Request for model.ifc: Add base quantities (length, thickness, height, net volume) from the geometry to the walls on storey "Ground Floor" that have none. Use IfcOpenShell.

First a look at what the model holds.

```python
import ifcopenshell
import ifcopenshell.util.element
import ifcopenshell.util.unit

model = ifcopenshell.open("model.ifc")
print(model.schema)
for unit_type in ("LENGTHUNIT", "AREAUNIT", "VOLUMEUNIT"):
    print(unit_type, ifcopenshell.util.unit.calculate_unit_scale(model, unit_type))
storey = next(s for s in model.by_type("IfcBuildingStorey") if s.Name == "Ground Floor")
walls = [e for e in ifcopenshell.util.element.get_decomposition(storey) if e.is_a("IfcWall")]
for e in sorted(walls, key=lambda e: e.id()):
    print(e.id(), e.is_a(), e.Name, list(ifcopenshell.util.element.get_psets(e, qtos_only=True)), sep=" | ")
```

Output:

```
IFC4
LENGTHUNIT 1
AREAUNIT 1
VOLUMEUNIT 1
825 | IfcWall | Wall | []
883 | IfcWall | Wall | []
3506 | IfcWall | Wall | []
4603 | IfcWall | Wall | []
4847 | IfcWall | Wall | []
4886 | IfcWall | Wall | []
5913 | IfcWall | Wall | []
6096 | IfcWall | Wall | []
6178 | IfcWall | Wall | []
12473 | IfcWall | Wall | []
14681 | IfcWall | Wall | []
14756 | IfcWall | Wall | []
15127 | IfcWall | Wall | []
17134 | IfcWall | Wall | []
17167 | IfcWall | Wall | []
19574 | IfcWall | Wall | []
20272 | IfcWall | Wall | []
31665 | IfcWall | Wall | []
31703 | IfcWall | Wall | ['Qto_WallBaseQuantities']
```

```python
import ifcopenshell
import ifcopenshell.api.pset
import ifcopenshell.geom
import ifcopenshell.util.element
import ifcopenshell.util.shape
import ifcopenshell.util.unit

model = ifcopenshell.open("model.ifc")
unit_scale = ifcopenshell.util.unit.calculate_unit_scale(model)
volume_scale = ifcopenshell.util.unit.calculate_unit_scale(model, "VOLUMEUNIT")
settings = ifcopenshell.geom.settings()

storey = next(s for s in model.by_type("IfcBuildingStorey") if s.Name == "Ground Floor")
walls = [e for e in ifcopenshell.util.element.get_decomposition(storey) if e.is_a("IfcWall")]

for e in sorted(walls, key=lambda e: e.id()):
    if ifcopenshell.util.element.get_psets(e, qtos_only=True, should_inherit=False):
        continue
    # Geometry comes back in metres, in the element's own axes.
    shape = ifcopenshell.geom.create_shape(settings, e)
    values = {
        "Length": ifcopenshell.util.shape.get_x(shape.geometry) / unit_scale,
        "Width": ifcopenshell.util.shape.get_y(shape.geometry) / unit_scale,
        "Height": ifcopenshell.util.shape.get_z(shape.geometry) / unit_scale,
        "NetVolume": ifcopenshell.util.shape.get_volume(shape.geometry) / volume_scale,
    }
    qto = ifcopenshell.api.pset.add_qto(model, product=e, name="Qto_WallBaseQuantities")
    ifcopenshell.api.pset.edit_qto(model, qto=qto, properties=values)
    print(e.id(), {k: round(v, 3) for k, v in values.items()})

model.write("model_updated.ifc")
```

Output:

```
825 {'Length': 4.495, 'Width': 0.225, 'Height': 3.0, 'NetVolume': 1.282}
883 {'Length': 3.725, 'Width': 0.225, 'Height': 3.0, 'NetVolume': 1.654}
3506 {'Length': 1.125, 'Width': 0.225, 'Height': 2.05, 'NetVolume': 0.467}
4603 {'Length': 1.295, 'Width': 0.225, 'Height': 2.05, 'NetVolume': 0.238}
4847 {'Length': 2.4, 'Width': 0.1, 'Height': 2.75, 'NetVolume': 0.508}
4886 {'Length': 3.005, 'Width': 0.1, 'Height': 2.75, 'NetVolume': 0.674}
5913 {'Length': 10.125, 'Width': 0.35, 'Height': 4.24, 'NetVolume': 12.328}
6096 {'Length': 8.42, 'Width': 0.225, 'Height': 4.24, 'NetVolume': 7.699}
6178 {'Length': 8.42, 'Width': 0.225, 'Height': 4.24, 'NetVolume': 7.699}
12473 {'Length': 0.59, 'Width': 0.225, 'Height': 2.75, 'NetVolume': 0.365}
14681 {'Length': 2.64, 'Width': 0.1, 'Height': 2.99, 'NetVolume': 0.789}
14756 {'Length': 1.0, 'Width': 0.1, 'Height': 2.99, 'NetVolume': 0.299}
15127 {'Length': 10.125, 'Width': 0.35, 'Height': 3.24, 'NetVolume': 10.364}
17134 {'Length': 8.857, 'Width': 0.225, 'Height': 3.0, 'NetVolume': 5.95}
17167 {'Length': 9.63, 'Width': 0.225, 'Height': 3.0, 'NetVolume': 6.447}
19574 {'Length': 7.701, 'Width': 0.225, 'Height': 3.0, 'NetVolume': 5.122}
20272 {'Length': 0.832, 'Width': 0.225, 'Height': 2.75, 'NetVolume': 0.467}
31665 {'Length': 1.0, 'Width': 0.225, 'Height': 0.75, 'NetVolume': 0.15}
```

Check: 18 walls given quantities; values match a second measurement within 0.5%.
